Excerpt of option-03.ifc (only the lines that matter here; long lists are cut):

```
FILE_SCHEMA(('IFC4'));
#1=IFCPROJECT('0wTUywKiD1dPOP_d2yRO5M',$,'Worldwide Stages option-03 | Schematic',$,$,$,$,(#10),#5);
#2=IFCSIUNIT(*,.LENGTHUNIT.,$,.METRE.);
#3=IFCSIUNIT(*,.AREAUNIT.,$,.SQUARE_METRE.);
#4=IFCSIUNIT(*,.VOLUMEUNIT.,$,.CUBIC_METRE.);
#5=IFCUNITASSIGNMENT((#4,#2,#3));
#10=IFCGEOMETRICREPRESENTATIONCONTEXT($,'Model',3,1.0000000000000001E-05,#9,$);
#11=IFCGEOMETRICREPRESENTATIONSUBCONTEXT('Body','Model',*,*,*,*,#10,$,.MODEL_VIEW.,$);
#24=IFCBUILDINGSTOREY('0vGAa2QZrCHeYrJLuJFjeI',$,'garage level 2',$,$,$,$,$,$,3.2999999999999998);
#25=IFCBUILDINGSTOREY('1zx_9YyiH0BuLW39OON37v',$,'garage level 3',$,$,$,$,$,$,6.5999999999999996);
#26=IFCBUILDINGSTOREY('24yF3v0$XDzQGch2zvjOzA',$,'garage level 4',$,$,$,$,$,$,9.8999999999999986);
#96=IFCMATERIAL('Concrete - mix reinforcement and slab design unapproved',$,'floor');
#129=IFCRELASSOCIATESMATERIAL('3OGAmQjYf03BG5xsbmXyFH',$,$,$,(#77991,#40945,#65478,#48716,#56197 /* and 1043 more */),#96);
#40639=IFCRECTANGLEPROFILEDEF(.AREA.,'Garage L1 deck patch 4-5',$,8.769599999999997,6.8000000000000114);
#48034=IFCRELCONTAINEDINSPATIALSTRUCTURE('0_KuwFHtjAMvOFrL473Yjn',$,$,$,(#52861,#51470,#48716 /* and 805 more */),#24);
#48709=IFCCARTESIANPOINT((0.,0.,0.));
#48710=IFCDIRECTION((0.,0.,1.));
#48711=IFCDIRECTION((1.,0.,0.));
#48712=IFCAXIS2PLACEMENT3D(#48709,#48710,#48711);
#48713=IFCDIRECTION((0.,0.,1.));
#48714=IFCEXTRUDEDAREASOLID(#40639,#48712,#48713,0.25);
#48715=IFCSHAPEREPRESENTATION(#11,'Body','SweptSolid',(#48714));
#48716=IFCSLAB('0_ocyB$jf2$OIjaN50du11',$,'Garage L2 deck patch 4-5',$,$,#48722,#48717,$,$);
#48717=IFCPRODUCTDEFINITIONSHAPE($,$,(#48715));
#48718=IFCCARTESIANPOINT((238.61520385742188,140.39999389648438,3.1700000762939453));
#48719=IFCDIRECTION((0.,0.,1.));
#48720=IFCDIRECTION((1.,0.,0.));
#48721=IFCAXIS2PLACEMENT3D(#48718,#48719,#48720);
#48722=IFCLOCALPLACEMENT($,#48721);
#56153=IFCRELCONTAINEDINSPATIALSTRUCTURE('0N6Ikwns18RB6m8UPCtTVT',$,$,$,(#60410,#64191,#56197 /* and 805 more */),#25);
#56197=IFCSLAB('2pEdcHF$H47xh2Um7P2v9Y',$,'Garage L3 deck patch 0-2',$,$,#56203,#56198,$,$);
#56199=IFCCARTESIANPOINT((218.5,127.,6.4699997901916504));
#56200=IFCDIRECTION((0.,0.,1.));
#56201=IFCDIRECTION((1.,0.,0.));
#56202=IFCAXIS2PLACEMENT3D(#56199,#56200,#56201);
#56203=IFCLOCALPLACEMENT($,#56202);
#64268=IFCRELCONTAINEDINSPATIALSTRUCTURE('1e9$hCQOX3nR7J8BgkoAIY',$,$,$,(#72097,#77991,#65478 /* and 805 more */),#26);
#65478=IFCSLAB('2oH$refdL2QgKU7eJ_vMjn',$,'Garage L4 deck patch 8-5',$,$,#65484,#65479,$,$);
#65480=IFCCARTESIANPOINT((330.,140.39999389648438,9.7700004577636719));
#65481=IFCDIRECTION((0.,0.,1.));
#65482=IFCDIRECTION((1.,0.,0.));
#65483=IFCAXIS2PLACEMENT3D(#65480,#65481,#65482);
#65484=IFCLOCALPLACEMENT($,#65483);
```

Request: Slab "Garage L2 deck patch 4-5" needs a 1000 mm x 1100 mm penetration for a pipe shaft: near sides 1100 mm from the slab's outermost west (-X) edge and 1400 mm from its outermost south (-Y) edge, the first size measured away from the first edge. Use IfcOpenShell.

```python
import numpy as np
import ifcopenshell
import ifcopenshell.api.feature
import ifcopenshell.api.geometry
import ifcopenshell.api.root
import ifcopenshell.geom
import ifcopenshell.util.placement
import ifcopenshell.util.representation
import ifcopenshell.util.shape
import ifcopenshell.util.unit

model = ifcopenshell.open("option-03.ifc")
unit_scale = ifcopenshell.util.unit.calculate_unit_scale(model)
settings = ifcopenshell.geom.settings()


def volume(element):
    """Net volume in cubic metres, openings subtracted."""
    shape = ifcopenshell.geom.create_shape(settings, element)
    return ifcopenshell.util.shape.get_volume(shape.geometry)


slab = model.by_guid("0_ocyB$jf2$OIjaN50du11")
before = volume(slab)

# Extent in the slab's own axes, in metres. The edges named are its -X and -Y sides.
slab_shape = ifcopenshell.geom.create_shape(settings, slab)
vertices = ifcopenshell.util.shape.get_vertices(slab_shape.geometry)
x_min, y_min, bottom = vertices.min(axis=0)
top = vertices[:, 2].max()

opening = ifcopenshell.api.root.create_entity(model, ifc_class="IfcOpeningElement", name="Pipe shaft opening", predefined_type="OPENING")
context = ifcopenshell.util.representation.get_context(model, "Model", "Body", "MODEL_VIEW")
width, depth = 1, 1.1
outline = [(0.0, 0.0), (width, 0.0), (width, depth), (0.0, depth), (0.0, 0.0)]
# Overshoot both faces by 50 mm so the cut is clean.
shape = ifcopenshell.api.geometry.add_slab_representation(
    model, context=context, depth=top - bottom + 0.1, polyline=outline
)
ifcopenshell.api.geometry.assign_representation(model, product=opening, representation=shape)

matrix = ifcopenshell.util.placement.get_local_placement(slab.ObjectPlacement)
matrix[:, 3] = matrix @ np.append(np.array([x_min + 1.1, y_min + 1.4, bottom - 0.05]) / unit_scale, 1.0)
ifcopenshell.api.geometry.edit_object_placement(model, product=opening, matrix=matrix, is_si=False)
ifcopenshell.api.feature.add_feature(model, feature=opening, element=slab)

after = volume(slab)

print(f"slab volume {before:.3f} -> {after:.3f} m3")

model.write("option-03_v2.ifc")
```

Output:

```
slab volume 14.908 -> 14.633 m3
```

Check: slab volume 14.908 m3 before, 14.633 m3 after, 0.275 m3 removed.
